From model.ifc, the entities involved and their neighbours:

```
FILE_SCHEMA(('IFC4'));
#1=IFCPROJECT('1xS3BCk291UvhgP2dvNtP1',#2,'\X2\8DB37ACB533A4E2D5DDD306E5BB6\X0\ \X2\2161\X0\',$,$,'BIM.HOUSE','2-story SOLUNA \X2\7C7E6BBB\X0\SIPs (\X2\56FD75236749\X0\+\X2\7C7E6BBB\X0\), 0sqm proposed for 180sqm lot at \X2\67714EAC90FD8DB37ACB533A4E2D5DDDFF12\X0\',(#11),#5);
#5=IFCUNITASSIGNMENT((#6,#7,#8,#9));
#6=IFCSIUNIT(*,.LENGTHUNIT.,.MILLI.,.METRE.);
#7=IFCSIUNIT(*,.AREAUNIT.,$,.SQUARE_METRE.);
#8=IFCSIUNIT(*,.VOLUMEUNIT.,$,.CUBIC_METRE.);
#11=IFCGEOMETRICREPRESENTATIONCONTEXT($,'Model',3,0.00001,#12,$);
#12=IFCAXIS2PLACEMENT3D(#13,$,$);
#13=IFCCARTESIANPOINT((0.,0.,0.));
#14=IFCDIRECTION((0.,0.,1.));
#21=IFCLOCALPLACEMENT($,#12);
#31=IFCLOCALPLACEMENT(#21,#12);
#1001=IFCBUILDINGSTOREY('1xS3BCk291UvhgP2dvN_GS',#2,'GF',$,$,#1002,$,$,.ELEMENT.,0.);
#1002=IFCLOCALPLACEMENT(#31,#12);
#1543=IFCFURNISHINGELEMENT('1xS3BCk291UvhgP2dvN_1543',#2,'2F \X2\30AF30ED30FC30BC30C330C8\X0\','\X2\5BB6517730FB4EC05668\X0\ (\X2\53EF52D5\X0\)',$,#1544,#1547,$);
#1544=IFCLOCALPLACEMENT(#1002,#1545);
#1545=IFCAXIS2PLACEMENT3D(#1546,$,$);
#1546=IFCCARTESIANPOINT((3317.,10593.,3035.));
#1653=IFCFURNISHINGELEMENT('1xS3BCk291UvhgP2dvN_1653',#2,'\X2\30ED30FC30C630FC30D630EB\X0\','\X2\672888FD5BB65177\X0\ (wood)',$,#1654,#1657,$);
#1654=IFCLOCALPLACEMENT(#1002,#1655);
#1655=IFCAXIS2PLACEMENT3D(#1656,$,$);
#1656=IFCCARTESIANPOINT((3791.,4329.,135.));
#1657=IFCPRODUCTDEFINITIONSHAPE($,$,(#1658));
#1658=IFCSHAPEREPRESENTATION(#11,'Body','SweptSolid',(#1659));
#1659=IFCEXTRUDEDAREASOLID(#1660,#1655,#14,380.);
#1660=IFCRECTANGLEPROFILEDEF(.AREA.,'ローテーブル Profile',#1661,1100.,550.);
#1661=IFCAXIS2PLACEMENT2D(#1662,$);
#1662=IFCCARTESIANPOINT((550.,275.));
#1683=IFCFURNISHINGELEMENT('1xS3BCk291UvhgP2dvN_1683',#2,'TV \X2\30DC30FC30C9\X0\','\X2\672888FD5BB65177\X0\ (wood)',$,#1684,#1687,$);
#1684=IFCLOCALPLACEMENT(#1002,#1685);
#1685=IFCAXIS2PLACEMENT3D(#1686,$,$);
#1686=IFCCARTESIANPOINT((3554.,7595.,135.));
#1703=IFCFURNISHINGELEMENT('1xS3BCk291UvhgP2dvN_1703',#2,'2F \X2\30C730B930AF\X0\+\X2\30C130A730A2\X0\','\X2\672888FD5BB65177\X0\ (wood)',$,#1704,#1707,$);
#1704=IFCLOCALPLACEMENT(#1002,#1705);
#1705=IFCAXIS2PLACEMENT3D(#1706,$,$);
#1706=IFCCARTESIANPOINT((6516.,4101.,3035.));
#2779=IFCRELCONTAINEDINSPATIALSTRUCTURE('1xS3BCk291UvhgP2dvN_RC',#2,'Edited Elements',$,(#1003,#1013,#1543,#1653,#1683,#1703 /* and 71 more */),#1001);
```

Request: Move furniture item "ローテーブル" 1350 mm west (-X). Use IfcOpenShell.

```python
import ifcopenshell
import ifcopenshell.api.geometry
import ifcopenshell.util.placement
import ifcopenshell.util.unit

model = ifcopenshell.open("model.ifc")
unit_scale = ifcopenshell.util.unit.calculate_unit_scale(model)

item = model.by_id(1653)
matrix = ifcopenshell.util.placement.get_local_placement(item.ObjectPlacement)
matrix[0, 3] -= 1.35 / unit_scale
ifcopenshell.api.geometry.edit_object_placement(model, product=item, matrix=matrix, is_si=False)

print(ifcopenshell.util.placement.get_local_placement(item.ObjectPlacement).round(3) + 0.0)

model.write("model_updated.ifc")
```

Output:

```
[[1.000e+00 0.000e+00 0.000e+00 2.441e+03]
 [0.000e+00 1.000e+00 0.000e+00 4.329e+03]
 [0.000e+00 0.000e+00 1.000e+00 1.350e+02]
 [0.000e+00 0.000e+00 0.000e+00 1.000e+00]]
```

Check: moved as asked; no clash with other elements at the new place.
